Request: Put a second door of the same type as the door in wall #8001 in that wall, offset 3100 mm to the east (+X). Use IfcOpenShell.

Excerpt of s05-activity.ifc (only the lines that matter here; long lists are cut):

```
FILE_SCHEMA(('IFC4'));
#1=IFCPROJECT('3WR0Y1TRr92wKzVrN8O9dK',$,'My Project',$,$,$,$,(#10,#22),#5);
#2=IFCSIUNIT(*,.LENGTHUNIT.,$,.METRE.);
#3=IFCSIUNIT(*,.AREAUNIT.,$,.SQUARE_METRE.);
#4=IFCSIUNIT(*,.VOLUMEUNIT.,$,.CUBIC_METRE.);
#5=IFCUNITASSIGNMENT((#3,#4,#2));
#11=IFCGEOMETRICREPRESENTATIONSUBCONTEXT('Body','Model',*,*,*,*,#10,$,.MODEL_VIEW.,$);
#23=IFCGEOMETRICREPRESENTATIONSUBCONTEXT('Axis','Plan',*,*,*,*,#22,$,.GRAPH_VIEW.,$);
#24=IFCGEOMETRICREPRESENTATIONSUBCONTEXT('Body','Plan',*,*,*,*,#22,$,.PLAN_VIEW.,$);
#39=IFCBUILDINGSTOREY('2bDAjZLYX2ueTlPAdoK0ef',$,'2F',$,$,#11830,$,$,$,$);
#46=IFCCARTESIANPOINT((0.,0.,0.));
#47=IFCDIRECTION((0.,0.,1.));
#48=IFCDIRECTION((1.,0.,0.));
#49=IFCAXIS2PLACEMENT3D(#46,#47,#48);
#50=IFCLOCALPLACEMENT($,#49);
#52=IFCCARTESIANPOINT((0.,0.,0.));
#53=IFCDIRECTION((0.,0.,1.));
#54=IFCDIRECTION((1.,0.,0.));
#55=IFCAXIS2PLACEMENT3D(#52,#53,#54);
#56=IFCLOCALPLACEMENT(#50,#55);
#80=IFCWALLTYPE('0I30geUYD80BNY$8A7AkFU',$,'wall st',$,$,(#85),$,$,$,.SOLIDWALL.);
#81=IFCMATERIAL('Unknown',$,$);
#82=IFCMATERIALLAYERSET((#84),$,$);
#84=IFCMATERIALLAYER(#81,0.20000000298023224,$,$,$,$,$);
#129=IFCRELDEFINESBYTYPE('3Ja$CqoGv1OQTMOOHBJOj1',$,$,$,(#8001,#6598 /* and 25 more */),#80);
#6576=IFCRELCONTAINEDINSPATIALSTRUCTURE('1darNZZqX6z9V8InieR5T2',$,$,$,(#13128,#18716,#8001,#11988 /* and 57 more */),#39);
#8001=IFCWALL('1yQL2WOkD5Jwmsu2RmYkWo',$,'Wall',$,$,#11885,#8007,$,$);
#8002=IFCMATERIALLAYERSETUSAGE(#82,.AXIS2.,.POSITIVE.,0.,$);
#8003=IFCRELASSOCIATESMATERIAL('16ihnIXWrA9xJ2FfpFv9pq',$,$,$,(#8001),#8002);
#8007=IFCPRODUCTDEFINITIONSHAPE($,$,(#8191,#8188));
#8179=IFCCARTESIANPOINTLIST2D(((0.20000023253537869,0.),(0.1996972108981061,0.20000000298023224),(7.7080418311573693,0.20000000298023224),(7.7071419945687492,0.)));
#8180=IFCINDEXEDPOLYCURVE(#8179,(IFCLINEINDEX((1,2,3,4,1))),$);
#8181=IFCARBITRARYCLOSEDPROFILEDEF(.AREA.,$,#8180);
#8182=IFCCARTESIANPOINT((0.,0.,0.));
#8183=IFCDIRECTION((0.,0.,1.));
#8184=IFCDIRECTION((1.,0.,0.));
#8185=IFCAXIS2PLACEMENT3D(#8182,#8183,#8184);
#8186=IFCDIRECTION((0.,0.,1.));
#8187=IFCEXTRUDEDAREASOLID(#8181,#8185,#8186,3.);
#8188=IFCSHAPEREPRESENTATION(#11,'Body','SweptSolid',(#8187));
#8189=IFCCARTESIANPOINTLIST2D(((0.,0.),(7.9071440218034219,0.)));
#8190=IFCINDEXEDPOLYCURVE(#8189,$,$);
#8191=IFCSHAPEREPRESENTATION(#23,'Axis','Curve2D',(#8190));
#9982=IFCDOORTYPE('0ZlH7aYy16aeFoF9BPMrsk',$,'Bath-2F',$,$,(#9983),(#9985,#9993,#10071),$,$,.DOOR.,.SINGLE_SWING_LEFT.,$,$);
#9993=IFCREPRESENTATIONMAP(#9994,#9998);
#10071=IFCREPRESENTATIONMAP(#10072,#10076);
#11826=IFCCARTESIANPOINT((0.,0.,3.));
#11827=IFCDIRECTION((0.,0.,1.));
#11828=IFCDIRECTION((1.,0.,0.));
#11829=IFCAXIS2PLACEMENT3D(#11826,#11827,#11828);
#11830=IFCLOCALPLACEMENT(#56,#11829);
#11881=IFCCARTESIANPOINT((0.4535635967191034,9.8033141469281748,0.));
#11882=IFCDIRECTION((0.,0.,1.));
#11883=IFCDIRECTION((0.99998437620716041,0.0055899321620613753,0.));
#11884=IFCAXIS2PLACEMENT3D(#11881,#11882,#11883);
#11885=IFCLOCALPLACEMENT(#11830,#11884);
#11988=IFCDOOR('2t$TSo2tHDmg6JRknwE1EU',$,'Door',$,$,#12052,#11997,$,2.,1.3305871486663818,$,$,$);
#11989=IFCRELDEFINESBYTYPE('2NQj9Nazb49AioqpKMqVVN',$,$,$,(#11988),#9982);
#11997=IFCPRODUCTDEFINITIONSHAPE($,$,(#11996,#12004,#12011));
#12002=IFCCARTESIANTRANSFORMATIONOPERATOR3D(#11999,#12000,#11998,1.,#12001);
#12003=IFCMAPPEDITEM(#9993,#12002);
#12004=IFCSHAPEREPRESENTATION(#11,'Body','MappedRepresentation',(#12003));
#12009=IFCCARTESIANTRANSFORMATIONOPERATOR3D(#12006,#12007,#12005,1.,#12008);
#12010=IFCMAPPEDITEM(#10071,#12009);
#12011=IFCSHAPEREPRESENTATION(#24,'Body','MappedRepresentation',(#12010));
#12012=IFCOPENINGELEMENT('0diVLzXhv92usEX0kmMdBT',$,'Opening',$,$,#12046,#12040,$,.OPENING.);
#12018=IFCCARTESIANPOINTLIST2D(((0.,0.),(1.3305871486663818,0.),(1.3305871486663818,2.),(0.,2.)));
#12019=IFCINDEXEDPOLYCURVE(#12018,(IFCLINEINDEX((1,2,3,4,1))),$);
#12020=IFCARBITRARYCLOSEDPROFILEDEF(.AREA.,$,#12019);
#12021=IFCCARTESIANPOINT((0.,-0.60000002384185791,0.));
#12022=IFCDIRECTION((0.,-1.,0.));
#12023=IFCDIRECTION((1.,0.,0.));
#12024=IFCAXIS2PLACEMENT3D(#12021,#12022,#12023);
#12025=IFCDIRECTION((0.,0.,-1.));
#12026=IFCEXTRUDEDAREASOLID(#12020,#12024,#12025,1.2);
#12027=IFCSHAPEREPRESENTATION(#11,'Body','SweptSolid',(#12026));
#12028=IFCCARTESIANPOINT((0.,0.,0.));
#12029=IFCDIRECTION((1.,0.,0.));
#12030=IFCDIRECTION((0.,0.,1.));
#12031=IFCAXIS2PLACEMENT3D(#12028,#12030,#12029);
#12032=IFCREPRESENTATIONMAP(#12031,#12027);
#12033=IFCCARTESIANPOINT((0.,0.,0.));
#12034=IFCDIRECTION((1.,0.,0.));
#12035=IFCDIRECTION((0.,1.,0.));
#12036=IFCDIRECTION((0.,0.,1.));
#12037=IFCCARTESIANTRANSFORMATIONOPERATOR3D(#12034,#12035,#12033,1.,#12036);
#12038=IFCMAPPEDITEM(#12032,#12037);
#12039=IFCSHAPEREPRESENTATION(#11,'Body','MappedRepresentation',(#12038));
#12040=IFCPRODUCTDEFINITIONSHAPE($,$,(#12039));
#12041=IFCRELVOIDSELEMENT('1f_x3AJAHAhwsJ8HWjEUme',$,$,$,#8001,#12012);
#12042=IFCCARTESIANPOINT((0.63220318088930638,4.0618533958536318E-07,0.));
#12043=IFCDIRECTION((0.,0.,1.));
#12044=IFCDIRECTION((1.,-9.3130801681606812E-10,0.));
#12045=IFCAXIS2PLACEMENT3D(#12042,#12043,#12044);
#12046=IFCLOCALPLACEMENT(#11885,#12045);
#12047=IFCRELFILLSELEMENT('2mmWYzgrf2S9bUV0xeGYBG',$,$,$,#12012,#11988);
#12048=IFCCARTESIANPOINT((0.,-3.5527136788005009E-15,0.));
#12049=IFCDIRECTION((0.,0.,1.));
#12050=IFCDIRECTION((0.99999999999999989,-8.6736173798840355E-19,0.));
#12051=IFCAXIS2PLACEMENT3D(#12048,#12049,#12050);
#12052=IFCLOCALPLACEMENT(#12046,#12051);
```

```python
import ifcopenshell
import ifcopenshell.api.feature
import ifcopenshell.api.geometry
import ifcopenshell.api.root
import ifcopenshell.geom
import ifcopenshell.util.element
import ifcopenshell.util.placement
import ifcopenshell.util.shape
import ifcopenshell.util.unit

model = ifcopenshell.open("s05-activity.ifc")
unit_scale = ifcopenshell.util.unit.calculate_unit_scale(model)
settings = ifcopenshell.geom.settings()


def volume(element):
    """Net volume in cubic metres, openings subtracted."""
    shape = ifcopenshell.geom.create_shape(settings, element)
    return ifcopenshell.util.shape.get_volume(shape.geometry)


door = model.by_id(11988)
opening = door.FillsVoids[0].RelatingOpeningElement
wall = opening.VoidsElements[0].RelatingBuildingElement
before = volume(wall)
shift = ifcopenshell.util.placement.get_local_placement(wall.ObjectPlacement)[:3, 0] * 3.1 / unit_scale

# copy_class copies the void relationship, type, container and properties, but no geometry.
new_opening = ifcopenshell.api.root.copy_class(model, product=opening)
new_opening.Representation = ifcopenshell.util.element.copy_deep(
    model, opening.Representation, exclude=["IfcGeometricRepresentationContext", "IfcRepresentationMap"]
)
new_door = ifcopenshell.api.root.copy_class(model, product=door)
new_door.Representation = ifcopenshell.util.element.copy_deep(
    model, door.Representation, exclude=["IfcGeometricRepresentationContext", "IfcRepresentationMap"]
)
ifcopenshell.api.feature.add_filling(model, opening=new_opening, element=new_door)

for old, new in ((opening, new_opening), (door, new_door)):
    matrix = ifcopenshell.util.placement.get_local_placement(old.ObjectPlacement)
    matrix[:3, 3] += shift
    ifcopenshell.api.geometry.edit_object_placement(model, product=new, matrix=matrix, is_si=False)

after = volume(wall)

print(f"wall volume {before:.3f} -> {after:.3f} m3")

model.write("s05-activity_edited.ifc")
```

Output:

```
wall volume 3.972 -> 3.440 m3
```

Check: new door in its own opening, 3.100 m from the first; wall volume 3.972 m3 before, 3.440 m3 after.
